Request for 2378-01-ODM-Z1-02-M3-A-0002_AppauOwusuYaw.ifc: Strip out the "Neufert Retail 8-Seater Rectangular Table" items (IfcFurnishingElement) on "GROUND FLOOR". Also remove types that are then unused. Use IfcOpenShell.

First a look at what the model holds.

```python
import ifcopenshell
import ifcopenshell.util.element

model = ifcopenshell.open("2378-01-ODM-Z1-02-M3-A-0002_AppauOwusuYaw.ifc")
print(model.schema)
storey = next(s for s in model.by_type("IfcBuildingStorey") if s.Name == "GROUND FLOOR")
furniture = [e for e in ifcopenshell.util.element.get_decomposition(storey) if e.is_a("IfcFurnishingElement")]
seen = {}
for e in furniture:
    element_type = ifcopenshell.util.element.get_type(e)
    name = element_type.Name if element_type not in (None, e) else None
    seen[name] = seen.get(name, 0) + 1
for name, count in sorted(seen.items(), key=str):
    print(count, "x", name)
```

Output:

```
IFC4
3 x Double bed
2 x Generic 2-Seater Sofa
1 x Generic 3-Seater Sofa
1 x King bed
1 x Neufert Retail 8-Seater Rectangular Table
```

```python
import ifcopenshell
import ifcopenshell.api.root
import ifcopenshell.util.element

model = ifcopenshell.open("2378-01-ODM-Z1-02-M3-A-0002_AppauOwusuYaw.ifc")

storey = next(s for s in model.by_type("IfcBuildingStorey") if s.Name == "GROUND FLOOR")
furniture = [e for e in ifcopenshell.util.element.get_decomposition(storey) if e.is_a("IfcFurnishingElement")]
targets = [e for e in furniture if (t := ifcopenshell.util.element.get_type(e)) not in (None, e) and t.Name == "Neufert Retail 8-Seater Rectangular Table"]
types = {ifcopenshell.util.element.get_type(e) for e in targets} - {None, *targets}

for e in targets:
    ifcopenshell.api.root.remove_product(model, product=e)
print(len(targets), "removed")

unused = [t for t in types if not ifcopenshell.util.element.get_types(t)]
for t in unused:
    ifcopenshell.api.root.remove_product(model, product=t)
print(len(unused), "unused types removed")

model.write("2378-01-ODM-Z1-02-M3-A-0002_AppauOwusuYaw_updated.ifc")
```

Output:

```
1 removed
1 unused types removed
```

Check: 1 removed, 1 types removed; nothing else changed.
